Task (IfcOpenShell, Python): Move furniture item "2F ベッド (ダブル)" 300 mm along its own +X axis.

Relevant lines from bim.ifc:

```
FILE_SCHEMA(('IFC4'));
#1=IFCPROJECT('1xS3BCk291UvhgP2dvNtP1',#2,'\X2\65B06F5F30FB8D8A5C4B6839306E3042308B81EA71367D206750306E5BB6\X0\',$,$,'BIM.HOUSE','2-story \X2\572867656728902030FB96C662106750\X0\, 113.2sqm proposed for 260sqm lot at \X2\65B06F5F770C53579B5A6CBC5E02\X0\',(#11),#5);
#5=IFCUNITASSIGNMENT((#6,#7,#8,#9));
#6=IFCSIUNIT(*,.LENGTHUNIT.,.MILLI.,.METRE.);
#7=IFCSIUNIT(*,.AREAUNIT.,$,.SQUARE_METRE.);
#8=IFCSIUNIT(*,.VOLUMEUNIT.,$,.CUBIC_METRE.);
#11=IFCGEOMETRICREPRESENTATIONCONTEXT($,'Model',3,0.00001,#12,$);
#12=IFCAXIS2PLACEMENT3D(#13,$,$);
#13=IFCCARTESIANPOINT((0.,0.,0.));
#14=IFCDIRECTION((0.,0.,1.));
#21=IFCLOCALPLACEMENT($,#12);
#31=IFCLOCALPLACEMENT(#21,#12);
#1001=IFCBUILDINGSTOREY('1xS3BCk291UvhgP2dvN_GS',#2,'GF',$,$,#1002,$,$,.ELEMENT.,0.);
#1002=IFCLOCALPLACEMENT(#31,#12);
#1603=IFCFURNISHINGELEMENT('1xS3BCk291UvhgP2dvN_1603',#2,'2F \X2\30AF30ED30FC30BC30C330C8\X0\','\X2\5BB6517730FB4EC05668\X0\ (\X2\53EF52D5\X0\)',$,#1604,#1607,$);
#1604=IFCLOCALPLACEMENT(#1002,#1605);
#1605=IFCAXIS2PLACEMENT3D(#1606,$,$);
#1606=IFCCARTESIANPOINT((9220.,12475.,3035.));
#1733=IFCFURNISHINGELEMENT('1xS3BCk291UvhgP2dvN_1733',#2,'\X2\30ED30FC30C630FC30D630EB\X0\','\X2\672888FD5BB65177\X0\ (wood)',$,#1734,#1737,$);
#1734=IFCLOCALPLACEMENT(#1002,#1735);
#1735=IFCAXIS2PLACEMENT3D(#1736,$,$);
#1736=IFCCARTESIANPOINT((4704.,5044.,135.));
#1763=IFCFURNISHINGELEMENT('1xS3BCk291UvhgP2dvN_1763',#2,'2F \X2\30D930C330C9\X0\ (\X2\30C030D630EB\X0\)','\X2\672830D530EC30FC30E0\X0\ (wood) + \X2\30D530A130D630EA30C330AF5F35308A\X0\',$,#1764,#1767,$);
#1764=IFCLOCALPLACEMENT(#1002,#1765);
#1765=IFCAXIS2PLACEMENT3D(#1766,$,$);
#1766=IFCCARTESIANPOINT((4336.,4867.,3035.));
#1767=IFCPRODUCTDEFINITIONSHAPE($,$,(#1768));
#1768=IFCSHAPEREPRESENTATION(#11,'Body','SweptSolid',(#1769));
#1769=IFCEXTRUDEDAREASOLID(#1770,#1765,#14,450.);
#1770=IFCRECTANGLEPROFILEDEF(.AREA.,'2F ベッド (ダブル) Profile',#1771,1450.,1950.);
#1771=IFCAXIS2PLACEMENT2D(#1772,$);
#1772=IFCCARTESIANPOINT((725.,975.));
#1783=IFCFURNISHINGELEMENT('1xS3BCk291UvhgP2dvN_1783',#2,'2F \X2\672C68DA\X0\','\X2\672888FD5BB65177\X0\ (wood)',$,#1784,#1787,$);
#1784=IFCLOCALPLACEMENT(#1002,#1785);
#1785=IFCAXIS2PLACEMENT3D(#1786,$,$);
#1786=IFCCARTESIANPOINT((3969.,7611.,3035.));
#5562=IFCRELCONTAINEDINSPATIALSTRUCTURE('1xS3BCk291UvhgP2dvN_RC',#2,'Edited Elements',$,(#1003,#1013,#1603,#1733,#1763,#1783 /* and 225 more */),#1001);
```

```python
import ifcopenshell
import ifcopenshell.api.geometry
import ifcopenshell.util.placement
import ifcopenshell.util.unit

model = ifcopenshell.open("bim.ifc")
unit_scale = ifcopenshell.util.unit.calculate_unit_scale(model)

item = model.by_guid("1xS3BCk291UvhgP2dvN_1763")
matrix = ifcopenshell.util.placement.get_local_placement(item.ObjectPlacement)
matrix[:3, 3] += matrix[:3, 0] * 0.3 / unit_scale
ifcopenshell.api.geometry.edit_object_placement(model, product=item, matrix=matrix, is_si=False)

print(ifcopenshell.util.placement.get_local_placement(item.ObjectPlacement).round(3) + 0.0)

model.write("bim_updated.ifc")
```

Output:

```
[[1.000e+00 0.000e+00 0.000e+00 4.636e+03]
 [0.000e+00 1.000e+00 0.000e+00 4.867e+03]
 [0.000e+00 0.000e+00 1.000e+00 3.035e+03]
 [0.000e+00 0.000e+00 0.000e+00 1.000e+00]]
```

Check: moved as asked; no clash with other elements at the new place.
